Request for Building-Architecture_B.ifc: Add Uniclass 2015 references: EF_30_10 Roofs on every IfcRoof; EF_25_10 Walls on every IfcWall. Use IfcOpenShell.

First a look at what the model holds.

```python
import ifcopenshell

model = ifcopenshell.open("Building-Architecture_B.ifc")
print(model.schema)
print("classifications:", [c.Name for c in model.by_type("IfcClassification")])
for ifc_class in ("IfcDoor", "IfcRoof", "IfcStair", "IfcWall", "IfcWindow"):
    print(ifc_class, len(model.by_type(ifc_class)))
```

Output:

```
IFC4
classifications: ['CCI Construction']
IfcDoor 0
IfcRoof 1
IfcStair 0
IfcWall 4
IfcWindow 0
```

```python
import ifcopenshell
import ifcopenshell.api.classification

model = ifcopenshell.open("Building-Architecture_B.ifc")

system = ifcopenshell.api.classification.add_classification(model, classification="Uniclass 2015")

codes = {
    "IfcRoof": ("EF_30_10", "Roofs"),
    "IfcWall": ("EF_25_10", "Walls"),
}
for ifc_class, (code, name) in codes.items():
    products = model.by_type(ifc_class)
    ifcopenshell.api.classification.add_reference(
        model, products=products, classification=system, identification=code, name=name
    )
    print(code, len(products))

model.write("Building-Architecture_B_rev.ifc")
```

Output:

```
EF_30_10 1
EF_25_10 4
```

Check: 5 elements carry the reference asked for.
